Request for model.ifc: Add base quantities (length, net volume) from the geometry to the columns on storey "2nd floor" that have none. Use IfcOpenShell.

First a look at what the model holds.

```python
import ifcopenshell
import ifcopenshell.util.element
import ifcopenshell.util.unit

model = ifcopenshell.open("model.ifc")
print(model.schema)
for unit_type in ("LENGTHUNIT", "AREAUNIT", "VOLUMEUNIT"):
    print(unit_type, ifcopenshell.util.unit.calculate_unit_scale(model, unit_type))
storey = next(s for s in model.by_type("IfcBuildingStorey") if s.Name == "2nd floor")
columns = [e for e in ifcopenshell.util.element.get_decomposition(storey) if e.is_a("IfcColumn")]
for e in sorted(columns, key=lambda e: e.id()):
    print(e.id(), e.is_a(), e.Name, list(ifcopenshell.util.element.get_psets(e, qtos_only=True)), sep=" | ")
```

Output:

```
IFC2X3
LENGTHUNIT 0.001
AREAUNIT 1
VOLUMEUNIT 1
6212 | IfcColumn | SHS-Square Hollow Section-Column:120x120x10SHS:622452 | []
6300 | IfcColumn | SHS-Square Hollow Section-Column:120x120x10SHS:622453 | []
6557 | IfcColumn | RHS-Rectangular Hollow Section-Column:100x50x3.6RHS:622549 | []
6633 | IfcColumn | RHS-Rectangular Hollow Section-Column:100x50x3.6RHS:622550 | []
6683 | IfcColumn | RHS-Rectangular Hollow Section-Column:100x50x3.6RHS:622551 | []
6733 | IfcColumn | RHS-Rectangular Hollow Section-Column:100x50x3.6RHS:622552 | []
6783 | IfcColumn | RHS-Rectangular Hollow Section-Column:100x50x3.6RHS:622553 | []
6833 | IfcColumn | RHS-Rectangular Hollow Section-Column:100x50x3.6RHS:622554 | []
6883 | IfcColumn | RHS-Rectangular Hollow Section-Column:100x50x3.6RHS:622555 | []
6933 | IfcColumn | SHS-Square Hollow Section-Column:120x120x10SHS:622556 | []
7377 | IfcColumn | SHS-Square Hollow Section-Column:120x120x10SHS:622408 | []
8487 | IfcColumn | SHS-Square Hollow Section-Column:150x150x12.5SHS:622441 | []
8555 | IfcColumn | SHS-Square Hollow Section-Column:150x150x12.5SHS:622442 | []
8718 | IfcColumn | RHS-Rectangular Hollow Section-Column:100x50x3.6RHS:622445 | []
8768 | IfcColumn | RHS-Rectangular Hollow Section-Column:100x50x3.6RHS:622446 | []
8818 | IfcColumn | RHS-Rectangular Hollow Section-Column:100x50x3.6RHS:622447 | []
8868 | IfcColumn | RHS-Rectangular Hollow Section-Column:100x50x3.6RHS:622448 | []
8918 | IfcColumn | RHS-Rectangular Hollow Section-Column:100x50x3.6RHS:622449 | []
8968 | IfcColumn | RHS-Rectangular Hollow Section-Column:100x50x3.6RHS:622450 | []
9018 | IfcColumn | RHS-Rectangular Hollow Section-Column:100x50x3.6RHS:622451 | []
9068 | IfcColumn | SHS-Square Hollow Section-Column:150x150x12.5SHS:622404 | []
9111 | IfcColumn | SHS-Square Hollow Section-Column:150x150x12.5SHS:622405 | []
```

```python
import ifcopenshell
import ifcopenshell.api.pset
import ifcopenshell.geom
import ifcopenshell.util.element
import ifcopenshell.util.shape
import ifcopenshell.util.unit

model = ifcopenshell.open("model.ifc")
unit_scale = ifcopenshell.util.unit.calculate_unit_scale(model)
volume_scale = ifcopenshell.util.unit.calculate_unit_scale(model, "VOLUMEUNIT")
settings = ifcopenshell.geom.settings()

storey = next(s for s in model.by_type("IfcBuildingStorey") if s.Name == "2nd floor")
columns = [e for e in ifcopenshell.util.element.get_decomposition(storey) if e.is_a("IfcColumn")]

for e in sorted(columns, key=lambda e: e.id()):
    if ifcopenshell.util.element.get_psets(e, qtos_only=True, should_inherit=False):
        continue
    # Geometry comes back in metres, in the element's own axes.
    shape = ifcopenshell.geom.create_shape(settings, e)
    values = {
        "Length": ifcopenshell.util.shape.get_z(shape.geometry) / unit_scale,
        "NetVolume": ifcopenshell.util.shape.get_volume(shape.geometry) / volume_scale,
    }
    qto = ifcopenshell.api.pset.add_qto(model, product=e, name="BaseQuantities")
    ifcopenshell.api.pset.edit_qto(model, qto=qto, properties=values)
    print(e.id(), {k: round(v, 3) for k, v in values.items()})

model.write("model_v2.ifc")
```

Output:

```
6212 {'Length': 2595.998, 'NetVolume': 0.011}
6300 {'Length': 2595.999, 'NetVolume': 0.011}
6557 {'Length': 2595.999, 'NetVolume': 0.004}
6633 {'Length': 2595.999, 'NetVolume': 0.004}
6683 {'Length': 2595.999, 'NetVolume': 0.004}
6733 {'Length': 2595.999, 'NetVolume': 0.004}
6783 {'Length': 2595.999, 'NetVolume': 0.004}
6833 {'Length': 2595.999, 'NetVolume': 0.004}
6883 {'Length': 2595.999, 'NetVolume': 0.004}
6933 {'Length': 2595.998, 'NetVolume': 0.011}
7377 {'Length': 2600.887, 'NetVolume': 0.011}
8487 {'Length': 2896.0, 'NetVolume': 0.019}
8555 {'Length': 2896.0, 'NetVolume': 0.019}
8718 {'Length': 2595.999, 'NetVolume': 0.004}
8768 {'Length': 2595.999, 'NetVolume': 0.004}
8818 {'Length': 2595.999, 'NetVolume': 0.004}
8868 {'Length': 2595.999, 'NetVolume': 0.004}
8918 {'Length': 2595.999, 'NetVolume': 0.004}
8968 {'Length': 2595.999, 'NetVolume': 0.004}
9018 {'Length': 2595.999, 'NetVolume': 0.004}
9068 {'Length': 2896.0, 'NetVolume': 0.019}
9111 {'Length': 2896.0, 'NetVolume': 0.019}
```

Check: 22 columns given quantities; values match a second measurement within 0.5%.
